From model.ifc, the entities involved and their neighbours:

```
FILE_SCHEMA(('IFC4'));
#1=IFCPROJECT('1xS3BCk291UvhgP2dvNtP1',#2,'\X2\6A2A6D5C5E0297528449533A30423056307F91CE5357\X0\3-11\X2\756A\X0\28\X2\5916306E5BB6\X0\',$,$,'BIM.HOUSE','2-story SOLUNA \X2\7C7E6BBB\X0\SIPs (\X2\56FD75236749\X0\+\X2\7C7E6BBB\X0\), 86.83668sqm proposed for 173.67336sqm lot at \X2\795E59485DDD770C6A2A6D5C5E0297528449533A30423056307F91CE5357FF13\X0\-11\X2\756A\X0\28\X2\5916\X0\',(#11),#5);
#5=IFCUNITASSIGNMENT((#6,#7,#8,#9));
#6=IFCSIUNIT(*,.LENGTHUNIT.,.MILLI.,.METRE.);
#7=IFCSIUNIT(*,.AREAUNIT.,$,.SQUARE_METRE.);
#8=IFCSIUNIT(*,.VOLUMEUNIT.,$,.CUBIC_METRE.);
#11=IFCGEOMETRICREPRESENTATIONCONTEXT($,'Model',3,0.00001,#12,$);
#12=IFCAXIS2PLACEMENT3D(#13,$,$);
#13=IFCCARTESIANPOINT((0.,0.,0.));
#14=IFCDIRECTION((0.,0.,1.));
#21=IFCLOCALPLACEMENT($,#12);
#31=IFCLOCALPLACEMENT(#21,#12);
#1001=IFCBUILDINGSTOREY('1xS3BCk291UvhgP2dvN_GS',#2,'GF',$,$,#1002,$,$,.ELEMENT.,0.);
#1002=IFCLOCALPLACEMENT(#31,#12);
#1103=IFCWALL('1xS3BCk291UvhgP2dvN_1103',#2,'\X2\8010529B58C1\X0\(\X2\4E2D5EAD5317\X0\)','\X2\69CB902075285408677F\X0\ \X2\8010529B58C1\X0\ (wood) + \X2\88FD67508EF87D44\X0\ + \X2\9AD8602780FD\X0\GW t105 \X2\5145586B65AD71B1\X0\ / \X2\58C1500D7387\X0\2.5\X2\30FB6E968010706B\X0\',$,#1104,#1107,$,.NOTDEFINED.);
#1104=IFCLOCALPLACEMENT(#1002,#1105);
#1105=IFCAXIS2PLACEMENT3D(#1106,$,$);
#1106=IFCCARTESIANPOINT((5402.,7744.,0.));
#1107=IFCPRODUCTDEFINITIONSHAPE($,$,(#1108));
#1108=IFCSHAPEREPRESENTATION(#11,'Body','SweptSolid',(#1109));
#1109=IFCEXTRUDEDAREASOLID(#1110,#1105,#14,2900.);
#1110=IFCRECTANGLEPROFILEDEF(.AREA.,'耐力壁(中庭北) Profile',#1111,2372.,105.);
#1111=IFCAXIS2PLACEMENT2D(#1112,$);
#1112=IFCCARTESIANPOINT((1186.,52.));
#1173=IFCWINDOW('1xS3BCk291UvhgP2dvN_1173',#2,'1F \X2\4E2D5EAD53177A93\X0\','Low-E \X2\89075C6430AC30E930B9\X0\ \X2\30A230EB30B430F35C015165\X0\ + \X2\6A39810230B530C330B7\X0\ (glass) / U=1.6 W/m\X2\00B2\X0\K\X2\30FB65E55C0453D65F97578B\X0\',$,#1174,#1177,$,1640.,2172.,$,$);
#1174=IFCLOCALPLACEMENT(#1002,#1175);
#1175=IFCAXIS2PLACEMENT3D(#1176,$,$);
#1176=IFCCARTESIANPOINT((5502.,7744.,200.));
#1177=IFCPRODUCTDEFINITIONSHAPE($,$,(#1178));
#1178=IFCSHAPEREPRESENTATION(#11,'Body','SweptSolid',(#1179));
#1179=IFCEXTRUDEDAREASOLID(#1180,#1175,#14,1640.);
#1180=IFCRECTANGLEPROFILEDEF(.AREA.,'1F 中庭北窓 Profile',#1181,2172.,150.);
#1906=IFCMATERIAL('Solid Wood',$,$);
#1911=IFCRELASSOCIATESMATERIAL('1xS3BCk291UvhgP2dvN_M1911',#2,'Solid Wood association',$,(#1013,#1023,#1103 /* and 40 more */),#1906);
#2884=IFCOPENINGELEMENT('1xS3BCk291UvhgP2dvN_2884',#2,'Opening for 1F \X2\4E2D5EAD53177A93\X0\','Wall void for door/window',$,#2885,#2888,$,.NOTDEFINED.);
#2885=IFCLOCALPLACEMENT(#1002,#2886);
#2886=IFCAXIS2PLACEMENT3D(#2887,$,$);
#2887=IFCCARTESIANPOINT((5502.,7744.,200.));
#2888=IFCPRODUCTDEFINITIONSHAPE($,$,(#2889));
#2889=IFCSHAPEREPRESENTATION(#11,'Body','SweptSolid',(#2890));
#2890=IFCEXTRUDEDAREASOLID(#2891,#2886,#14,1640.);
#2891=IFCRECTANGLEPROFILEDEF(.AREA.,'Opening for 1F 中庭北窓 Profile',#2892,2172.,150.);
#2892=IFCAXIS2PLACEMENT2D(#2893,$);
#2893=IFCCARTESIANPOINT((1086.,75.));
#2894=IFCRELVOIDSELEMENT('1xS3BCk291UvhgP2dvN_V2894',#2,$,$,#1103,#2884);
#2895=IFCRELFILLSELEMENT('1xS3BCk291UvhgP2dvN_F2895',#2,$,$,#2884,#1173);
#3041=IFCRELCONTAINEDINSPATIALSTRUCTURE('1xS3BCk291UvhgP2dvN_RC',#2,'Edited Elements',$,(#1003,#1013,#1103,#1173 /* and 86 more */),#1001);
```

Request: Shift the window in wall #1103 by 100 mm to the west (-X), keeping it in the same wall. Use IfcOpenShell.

```python
import ifcopenshell
import ifcopenshell.api.geometry
import ifcopenshell.util.placement
import ifcopenshell.util.unit

model = ifcopenshell.open("model.ifc")
unit_scale = ifcopenshell.util.unit.calculate_unit_scale(model)

window = model.by_id(1173)
opening = window.FillsVoids[0].RelatingOpeningElement
wall = opening.VoidsElements[0].RelatingBuildingElement

wall_matrix = ifcopenshell.util.placement.get_local_placement(wall.ObjectPlacement)
shift = wall_matrix[:3, 0] * -0.1 / unit_scale
before = ifcopenshell.util.placement.get_local_placement(window.ObjectPlacement)[:3, 3].copy()

# The window is not placed relative to its opening, so move both.
for product in (opening, window):
    matrix = ifcopenshell.util.placement.get_local_placement(product.ObjectPlacement)
    matrix[:3, 3] += shift
    ifcopenshell.api.geometry.edit_object_placement(model, product=product, matrix=matrix, is_si=False)

after = ifcopenshell.util.placement.get_local_placement(window.ObjectPlacement)[:3, 3]
print("window moved by", (after - before).round(3) + 0.0)

model.write("model_updated.ifc")
```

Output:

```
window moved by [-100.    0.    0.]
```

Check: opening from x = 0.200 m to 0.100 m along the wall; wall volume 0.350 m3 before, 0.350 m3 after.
